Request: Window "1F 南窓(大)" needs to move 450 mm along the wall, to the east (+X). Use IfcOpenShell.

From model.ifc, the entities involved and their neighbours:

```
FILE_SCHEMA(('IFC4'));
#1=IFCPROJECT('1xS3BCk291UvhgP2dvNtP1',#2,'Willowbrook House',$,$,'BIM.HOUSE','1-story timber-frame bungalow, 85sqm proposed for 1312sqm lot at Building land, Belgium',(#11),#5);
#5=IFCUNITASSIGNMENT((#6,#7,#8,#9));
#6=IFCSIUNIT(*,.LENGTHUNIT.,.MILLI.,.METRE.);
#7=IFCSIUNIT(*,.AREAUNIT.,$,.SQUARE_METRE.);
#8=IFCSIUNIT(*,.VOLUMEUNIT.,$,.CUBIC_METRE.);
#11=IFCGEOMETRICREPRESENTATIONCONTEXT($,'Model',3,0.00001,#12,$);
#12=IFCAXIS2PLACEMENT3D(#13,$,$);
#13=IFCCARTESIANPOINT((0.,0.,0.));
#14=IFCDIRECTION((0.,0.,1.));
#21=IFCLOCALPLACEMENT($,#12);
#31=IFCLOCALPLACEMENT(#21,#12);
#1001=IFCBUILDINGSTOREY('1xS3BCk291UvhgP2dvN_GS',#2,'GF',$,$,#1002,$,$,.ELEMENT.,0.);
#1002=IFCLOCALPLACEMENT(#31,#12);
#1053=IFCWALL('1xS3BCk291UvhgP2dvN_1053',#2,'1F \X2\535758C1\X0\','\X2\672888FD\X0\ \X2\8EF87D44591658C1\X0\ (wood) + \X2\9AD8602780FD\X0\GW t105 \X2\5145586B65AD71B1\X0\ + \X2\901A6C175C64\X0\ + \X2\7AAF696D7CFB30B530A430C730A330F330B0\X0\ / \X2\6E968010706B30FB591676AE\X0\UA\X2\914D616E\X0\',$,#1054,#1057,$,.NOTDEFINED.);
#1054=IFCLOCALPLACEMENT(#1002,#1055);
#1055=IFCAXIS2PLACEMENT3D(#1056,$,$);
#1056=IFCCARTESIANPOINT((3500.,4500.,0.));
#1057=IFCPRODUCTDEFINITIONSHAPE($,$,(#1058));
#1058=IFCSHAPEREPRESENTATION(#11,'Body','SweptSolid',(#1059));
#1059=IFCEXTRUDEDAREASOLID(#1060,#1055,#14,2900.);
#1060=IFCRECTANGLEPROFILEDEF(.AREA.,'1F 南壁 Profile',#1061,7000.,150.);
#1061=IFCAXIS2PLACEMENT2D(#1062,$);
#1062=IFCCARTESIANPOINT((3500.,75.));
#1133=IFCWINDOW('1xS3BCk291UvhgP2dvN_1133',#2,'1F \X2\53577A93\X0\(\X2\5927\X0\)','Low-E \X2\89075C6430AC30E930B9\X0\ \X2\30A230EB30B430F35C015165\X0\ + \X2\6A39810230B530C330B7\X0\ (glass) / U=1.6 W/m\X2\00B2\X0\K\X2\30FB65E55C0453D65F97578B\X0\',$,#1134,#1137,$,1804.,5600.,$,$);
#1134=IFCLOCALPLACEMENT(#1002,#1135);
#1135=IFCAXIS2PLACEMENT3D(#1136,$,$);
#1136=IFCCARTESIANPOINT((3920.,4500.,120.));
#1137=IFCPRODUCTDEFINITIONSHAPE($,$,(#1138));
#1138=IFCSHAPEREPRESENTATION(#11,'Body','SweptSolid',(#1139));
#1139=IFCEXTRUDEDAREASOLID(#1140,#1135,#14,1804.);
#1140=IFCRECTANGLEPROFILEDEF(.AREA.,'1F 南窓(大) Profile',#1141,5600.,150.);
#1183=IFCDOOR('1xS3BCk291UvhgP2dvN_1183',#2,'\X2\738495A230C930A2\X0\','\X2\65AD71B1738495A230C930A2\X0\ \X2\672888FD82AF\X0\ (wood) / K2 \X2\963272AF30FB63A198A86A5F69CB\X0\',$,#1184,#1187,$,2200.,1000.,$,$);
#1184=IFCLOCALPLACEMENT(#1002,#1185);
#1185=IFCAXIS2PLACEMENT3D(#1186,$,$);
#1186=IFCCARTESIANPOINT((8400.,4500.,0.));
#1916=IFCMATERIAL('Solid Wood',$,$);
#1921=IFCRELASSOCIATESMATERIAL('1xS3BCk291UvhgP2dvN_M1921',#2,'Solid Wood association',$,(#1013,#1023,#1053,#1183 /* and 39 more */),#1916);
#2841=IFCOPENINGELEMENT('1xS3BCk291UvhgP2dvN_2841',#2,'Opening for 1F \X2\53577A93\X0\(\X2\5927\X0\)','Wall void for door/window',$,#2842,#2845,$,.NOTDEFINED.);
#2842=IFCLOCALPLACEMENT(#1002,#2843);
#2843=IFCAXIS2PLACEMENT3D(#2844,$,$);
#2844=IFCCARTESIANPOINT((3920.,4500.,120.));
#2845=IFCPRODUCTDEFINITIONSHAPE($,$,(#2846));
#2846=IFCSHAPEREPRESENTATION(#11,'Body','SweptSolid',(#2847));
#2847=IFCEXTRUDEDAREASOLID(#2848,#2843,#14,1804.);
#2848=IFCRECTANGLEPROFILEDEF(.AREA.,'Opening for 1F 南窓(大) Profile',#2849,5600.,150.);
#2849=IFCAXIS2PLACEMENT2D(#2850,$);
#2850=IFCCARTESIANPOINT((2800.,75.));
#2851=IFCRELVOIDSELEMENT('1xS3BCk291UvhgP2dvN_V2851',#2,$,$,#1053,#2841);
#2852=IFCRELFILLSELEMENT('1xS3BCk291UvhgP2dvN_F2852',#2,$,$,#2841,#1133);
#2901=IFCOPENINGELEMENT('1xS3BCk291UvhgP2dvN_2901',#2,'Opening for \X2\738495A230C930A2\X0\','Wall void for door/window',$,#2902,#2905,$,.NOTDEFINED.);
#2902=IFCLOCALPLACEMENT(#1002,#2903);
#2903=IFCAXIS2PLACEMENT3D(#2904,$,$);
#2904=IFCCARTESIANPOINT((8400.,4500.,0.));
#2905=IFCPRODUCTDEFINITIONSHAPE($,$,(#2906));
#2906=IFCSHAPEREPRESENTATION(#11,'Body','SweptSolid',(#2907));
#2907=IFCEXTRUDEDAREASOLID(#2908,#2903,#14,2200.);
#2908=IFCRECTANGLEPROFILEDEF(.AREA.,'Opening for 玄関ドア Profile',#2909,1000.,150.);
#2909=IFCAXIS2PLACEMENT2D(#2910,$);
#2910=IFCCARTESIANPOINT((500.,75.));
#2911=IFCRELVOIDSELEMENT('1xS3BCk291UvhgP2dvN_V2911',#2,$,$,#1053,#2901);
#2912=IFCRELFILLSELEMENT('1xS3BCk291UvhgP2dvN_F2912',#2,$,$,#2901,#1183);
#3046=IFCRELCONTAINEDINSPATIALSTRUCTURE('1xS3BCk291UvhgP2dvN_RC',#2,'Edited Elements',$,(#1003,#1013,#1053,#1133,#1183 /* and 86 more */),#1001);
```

```python
import ifcopenshell
import ifcopenshell.api.geometry
import ifcopenshell.util.placement
import ifcopenshell.util.unit

model = ifcopenshell.open("model.ifc")
unit_scale = ifcopenshell.util.unit.calculate_unit_scale(model)

window = model.by_guid("1xS3BCk291UvhgP2dvN_1133")
opening = window.FillsVoids[0].RelatingOpeningElement
wall = opening.VoidsElements[0].RelatingBuildingElement

wall_matrix = ifcopenshell.util.placement.get_local_placement(wall.ObjectPlacement)
shift = wall_matrix[:3, 0] * 0.45 / unit_scale
before = ifcopenshell.util.placement.get_local_placement(window.ObjectPlacement)[:3, 3].copy()

# The window is not placed relative to its opening, so move both.
for product in (opening, window):
    matrix = ifcopenshell.util.placement.get_local_placement(product.ObjectPlacement)
    matrix[:3, 3] += shift
    ifcopenshell.api.geometry.edit_object_placement(model, product=product, matrix=matrix, is_si=False)

after = ifcopenshell.util.placement.get_local_placement(window.ObjectPlacement)[:3, 3]
print("window moved by", (after - before).round(3) + 0.0)

model.write("model-out.ifc")
```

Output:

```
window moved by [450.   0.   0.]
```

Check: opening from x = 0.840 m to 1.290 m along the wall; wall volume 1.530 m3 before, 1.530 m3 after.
